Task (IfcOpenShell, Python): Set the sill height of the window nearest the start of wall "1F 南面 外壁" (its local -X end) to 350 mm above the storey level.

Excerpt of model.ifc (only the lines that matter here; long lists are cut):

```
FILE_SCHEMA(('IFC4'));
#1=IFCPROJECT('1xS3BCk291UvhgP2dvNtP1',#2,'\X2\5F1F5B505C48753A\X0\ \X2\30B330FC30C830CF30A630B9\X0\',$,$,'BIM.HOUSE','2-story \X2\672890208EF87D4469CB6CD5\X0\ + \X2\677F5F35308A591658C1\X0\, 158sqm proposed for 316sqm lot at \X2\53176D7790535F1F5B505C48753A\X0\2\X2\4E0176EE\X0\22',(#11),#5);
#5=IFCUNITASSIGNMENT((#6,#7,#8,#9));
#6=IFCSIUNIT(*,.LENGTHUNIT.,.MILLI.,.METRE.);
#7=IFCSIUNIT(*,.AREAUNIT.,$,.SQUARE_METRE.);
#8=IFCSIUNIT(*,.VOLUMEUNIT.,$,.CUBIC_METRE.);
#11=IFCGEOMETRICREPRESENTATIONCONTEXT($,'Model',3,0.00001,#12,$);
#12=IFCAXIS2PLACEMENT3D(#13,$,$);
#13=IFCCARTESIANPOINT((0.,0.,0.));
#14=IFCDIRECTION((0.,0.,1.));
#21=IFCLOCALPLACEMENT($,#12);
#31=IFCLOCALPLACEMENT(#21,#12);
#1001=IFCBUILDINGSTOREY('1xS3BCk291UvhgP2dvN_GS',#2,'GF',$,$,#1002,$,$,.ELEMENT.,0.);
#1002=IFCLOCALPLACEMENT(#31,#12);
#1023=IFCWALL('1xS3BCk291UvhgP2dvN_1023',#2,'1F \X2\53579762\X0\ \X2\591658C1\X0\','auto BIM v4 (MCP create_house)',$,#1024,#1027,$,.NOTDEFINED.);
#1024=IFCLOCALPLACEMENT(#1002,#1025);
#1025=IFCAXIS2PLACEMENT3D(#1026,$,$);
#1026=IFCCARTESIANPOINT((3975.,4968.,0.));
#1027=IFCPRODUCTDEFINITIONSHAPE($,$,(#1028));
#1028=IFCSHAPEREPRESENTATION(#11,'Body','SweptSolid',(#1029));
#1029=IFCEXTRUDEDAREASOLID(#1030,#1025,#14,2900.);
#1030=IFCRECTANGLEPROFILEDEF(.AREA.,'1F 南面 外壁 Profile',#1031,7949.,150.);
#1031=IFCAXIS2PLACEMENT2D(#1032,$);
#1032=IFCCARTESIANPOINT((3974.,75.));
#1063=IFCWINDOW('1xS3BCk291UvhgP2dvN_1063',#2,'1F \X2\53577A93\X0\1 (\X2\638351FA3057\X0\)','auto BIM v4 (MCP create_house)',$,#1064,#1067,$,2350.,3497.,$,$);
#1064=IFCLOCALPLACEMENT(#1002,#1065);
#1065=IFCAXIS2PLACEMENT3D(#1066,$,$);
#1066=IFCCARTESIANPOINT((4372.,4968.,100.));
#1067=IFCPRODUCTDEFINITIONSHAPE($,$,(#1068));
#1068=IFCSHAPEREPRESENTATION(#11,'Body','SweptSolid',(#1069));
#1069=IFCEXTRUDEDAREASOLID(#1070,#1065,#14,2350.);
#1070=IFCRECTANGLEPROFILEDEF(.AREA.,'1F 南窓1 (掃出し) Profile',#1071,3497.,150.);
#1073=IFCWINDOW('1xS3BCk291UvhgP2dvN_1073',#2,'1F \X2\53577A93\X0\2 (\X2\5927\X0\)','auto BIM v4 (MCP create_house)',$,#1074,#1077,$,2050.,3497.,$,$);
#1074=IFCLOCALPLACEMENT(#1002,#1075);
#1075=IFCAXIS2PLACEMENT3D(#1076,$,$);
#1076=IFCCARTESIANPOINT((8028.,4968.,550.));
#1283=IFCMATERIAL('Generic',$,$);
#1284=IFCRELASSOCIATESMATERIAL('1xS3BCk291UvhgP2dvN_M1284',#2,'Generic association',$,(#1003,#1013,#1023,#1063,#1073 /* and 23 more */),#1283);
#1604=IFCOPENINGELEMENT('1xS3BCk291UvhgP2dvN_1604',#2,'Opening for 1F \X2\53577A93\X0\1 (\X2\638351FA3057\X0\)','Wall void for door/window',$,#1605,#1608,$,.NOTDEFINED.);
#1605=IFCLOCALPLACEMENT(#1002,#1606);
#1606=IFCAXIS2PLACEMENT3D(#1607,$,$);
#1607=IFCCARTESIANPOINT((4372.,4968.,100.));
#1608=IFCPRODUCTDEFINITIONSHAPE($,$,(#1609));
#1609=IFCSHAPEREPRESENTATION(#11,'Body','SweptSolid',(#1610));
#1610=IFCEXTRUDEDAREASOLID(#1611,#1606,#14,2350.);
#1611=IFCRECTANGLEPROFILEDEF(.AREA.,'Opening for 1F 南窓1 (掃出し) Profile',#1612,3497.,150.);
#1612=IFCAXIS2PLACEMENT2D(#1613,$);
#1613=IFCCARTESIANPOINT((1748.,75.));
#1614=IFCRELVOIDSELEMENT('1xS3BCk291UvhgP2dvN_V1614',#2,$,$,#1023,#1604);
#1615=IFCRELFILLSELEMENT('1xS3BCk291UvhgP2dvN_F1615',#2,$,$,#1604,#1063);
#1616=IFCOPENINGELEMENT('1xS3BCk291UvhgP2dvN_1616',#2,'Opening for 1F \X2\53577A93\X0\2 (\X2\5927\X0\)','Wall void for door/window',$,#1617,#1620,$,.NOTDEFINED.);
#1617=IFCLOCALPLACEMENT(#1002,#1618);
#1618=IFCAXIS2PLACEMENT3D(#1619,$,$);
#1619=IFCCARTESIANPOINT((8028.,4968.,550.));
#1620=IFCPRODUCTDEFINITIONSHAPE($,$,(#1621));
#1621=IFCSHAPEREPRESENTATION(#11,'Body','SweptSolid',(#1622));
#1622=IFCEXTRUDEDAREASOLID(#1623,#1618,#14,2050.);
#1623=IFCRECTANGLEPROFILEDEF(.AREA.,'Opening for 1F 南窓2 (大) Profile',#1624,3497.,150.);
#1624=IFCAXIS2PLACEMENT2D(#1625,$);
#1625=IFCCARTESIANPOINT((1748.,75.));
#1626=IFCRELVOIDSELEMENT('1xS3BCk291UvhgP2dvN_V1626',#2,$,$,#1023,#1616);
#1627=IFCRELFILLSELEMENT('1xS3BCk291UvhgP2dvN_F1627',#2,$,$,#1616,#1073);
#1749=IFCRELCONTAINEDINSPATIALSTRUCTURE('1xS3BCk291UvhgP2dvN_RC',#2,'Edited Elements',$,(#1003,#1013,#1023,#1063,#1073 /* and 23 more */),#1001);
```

```python
import numpy as np
import ifcopenshell
import ifcopenshell.api.geometry
import ifcopenshell.geom
import ifcopenshell.util.element
import ifcopenshell.util.placement
import ifcopenshell.util.shape
import ifcopenshell.util.unit

model = ifcopenshell.open("model.ifc")
unit_scale = ifcopenshell.util.unit.calculate_unit_scale(model)

window = model.by_guid("1xS3BCk291UvhgP2dvN_1063")
opening = window.FillsVoids[0].RelatingOpeningElement
storey = ifcopenshell.util.element.get_container(window, ifc_class="IfcBuildingStorey")
level = ifcopenshell.util.placement.get_local_placement(storey.ObjectPlacement)[2, 3]

# The opening's origin need not be at the sill, so measure its lowest point.
shape = ifcopenshell.geom.create_shape(ifcopenshell.geom.settings(), opening)
bottom = ifcopenshell.util.shape.get_shape_bottom_elevation(shape, shape.geometry) / unit_scale
dz = level + 350.0 - bottom

shift = np.array([0.0, 0.0, dz])
# The window is not placed relative to its opening, so move both.
for product in (opening, window):
    matrix = ifcopenshell.util.placement.get_local_placement(product.ObjectPlacement)
    matrix[:3, 3] += shift
    ifcopenshell.api.geometry.edit_object_placement(model, product=product, matrix=matrix, is_si=False)

print(f"moved by {dz * unit_scale:+.3f} m")

model.write("model_v2.ifc")
```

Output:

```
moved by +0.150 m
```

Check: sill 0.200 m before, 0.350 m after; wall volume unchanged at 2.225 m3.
